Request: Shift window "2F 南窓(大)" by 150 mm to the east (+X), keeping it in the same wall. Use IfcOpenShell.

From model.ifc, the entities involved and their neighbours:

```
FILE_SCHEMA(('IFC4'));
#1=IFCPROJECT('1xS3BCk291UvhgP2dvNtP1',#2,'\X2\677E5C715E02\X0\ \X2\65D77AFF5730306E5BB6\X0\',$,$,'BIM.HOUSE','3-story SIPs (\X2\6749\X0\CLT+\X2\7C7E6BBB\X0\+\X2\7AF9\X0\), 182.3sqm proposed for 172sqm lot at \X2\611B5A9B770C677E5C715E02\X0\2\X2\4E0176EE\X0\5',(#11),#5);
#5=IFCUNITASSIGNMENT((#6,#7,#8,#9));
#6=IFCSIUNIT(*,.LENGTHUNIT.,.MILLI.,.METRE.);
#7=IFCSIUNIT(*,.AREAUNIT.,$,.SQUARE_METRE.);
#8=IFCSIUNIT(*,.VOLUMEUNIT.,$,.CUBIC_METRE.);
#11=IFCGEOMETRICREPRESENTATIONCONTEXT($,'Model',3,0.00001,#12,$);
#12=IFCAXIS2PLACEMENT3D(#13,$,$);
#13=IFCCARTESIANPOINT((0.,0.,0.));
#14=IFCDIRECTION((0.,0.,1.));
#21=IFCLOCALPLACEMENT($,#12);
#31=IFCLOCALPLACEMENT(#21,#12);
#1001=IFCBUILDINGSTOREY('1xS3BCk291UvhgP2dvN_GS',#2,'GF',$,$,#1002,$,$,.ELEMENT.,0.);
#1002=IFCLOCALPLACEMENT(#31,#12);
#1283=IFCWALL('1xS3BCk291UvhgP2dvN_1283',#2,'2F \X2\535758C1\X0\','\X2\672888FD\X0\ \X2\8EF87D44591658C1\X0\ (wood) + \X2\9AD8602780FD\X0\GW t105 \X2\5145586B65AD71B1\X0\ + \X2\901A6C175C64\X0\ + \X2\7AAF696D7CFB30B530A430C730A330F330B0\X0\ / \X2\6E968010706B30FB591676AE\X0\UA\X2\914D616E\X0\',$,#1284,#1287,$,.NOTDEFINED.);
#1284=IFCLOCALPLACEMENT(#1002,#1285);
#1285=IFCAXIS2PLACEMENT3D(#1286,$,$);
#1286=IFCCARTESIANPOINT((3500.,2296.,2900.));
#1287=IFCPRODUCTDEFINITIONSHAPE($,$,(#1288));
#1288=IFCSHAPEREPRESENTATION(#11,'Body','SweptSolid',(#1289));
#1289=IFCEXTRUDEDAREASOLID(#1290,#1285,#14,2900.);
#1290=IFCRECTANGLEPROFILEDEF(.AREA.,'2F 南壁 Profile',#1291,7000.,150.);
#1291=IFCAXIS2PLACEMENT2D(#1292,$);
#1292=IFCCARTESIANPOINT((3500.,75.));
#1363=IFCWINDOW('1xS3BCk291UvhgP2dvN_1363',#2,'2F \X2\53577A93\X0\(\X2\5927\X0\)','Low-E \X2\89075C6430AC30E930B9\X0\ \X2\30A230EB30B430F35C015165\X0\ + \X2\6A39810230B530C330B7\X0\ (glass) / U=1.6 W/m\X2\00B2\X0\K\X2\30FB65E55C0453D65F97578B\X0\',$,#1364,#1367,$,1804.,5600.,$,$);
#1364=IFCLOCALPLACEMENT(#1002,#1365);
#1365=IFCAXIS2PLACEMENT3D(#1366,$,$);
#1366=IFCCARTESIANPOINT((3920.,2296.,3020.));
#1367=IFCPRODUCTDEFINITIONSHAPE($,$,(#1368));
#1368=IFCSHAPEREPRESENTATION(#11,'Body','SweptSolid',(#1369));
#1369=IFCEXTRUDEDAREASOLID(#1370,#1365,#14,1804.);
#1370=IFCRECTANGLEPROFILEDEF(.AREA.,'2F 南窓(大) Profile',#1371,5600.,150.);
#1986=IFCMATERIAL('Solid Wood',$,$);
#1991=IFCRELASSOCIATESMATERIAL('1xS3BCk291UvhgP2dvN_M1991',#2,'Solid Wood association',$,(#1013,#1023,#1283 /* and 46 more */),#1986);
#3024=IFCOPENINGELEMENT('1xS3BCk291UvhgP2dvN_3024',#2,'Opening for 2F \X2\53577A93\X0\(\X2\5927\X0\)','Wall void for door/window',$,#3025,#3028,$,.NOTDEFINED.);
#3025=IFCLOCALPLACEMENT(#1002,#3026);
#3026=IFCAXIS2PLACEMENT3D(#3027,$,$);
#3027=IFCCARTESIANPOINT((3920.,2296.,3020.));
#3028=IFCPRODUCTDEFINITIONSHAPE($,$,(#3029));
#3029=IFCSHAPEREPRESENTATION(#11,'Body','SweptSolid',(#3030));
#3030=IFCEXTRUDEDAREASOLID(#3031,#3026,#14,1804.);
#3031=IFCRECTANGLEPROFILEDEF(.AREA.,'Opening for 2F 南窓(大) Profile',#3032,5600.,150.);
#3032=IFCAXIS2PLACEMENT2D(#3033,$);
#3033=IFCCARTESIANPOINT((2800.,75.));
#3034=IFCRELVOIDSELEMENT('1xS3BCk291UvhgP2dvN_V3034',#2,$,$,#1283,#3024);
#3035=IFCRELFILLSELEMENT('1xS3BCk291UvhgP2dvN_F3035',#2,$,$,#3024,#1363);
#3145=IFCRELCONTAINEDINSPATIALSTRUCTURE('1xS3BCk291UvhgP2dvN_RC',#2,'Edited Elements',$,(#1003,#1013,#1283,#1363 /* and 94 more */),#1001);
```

```python
import ifcopenshell
import ifcopenshell.api.geometry
import ifcopenshell.util.placement
import ifcopenshell.util.unit

model = ifcopenshell.open("model.ifc")
unit_scale = ifcopenshell.util.unit.calculate_unit_scale(model)

window = model.by_guid("1xS3BCk291UvhgP2dvN_1363")
opening = window.FillsVoids[0].RelatingOpeningElement
wall = opening.VoidsElements[0].RelatingBuildingElement

wall_matrix = ifcopenshell.util.placement.get_local_placement(wall.ObjectPlacement)
shift = wall_matrix[:3, 0] * 0.15 / unit_scale
before = ifcopenshell.util.placement.get_local_placement(window.ObjectPlacement)[:3, 3].copy()

# The window is not placed relative to its opening, so move both.
for product in (opening, window):
    matrix = ifcopenshell.util.placement.get_local_placement(product.ObjectPlacement)
    matrix[:3, 3] += shift
    ifcopenshell.api.geometry.edit_object_placement(model, product=product, matrix=matrix, is_si=False)

after = ifcopenshell.util.placement.get_local_placement(window.ObjectPlacement)[:3, 3]
print("window moved by", (after - before).round(3) + 0.0)

model.write("model_v2.ifc")
```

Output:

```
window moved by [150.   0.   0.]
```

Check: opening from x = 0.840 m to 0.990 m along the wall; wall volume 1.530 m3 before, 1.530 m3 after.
